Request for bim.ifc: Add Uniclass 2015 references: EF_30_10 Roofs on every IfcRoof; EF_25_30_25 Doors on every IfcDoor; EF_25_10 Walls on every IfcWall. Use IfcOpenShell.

First a look at what the model holds.

```python
import ifcopenshell

model = ifcopenshell.open("bim.ifc")
print(model.schema)
print("classifications:", [c.Name for c in model.by_type("IfcClassification")])
for ifc_class in ("IfcDoor", "IfcRoof", "IfcStair", "IfcWall", "IfcWindow"):
    print(ifc_class, len(model.by_type(ifc_class)))
```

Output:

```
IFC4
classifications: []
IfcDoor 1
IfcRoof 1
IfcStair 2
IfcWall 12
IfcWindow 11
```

```python
import ifcopenshell
import ifcopenshell.api.classification

model = ifcopenshell.open("bim.ifc")

system = ifcopenshell.api.classification.add_classification(model, classification="Uniclass 2015")

codes = {
    "IfcRoof": ("EF_30_10", "Roofs"),
    "IfcDoor": ("EF_25_30_25", "Doors"),
    "IfcWall": ("EF_25_10", "Walls"),
}
for ifc_class, (code, name) in codes.items():
    products = model.by_type(ifc_class)
    ifcopenshell.api.classification.add_reference(
        model, products=products, classification=system, identification=code, name=name
    )
    print(code, len(products))

model.write("bim_rev.ifc")
```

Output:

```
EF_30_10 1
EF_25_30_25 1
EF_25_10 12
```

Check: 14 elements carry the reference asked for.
